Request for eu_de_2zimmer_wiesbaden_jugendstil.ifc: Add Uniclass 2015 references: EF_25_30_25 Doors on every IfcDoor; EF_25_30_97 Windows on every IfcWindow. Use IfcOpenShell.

First a look at what the model holds.

```python
import ifcopenshell

model = ifcopenshell.open("eu_de_2zimmer_wiesbaden_jugendstil.ifc")
print(model.schema)
print("classifications:", [c.Name for c in model.by_type("IfcClassification")])
for ifc_class in ("IfcDoor", "IfcRoof", "IfcStair", "IfcWall", "IfcWindow"):
    print(ifc_class, len(model.by_type(ifc_class)))
```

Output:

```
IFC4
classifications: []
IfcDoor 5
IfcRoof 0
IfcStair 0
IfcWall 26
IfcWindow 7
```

```python
import ifcopenshell
import ifcopenshell.api.classification

model = ifcopenshell.open("eu_de_2zimmer_wiesbaden_jugendstil.ifc")

system = ifcopenshell.api.classification.add_classification(model, classification="Uniclass 2015")

codes = {
    "IfcDoor": ("EF_25_30_25", "Doors"),
    "IfcWindow": ("EF_25_30_97", "Windows"),
}
for ifc_class, (code, name) in codes.items():
    products = model.by_type(ifc_class)
    ifcopenshell.api.classification.add_reference(
        model, products=products, classification=system, identification=code, name=name
    )
    print(code, len(products))

model.write("eu_de_2zimmer_wiesbaden_jugendstil_edited.ifc")
```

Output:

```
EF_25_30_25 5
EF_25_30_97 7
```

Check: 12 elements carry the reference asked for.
